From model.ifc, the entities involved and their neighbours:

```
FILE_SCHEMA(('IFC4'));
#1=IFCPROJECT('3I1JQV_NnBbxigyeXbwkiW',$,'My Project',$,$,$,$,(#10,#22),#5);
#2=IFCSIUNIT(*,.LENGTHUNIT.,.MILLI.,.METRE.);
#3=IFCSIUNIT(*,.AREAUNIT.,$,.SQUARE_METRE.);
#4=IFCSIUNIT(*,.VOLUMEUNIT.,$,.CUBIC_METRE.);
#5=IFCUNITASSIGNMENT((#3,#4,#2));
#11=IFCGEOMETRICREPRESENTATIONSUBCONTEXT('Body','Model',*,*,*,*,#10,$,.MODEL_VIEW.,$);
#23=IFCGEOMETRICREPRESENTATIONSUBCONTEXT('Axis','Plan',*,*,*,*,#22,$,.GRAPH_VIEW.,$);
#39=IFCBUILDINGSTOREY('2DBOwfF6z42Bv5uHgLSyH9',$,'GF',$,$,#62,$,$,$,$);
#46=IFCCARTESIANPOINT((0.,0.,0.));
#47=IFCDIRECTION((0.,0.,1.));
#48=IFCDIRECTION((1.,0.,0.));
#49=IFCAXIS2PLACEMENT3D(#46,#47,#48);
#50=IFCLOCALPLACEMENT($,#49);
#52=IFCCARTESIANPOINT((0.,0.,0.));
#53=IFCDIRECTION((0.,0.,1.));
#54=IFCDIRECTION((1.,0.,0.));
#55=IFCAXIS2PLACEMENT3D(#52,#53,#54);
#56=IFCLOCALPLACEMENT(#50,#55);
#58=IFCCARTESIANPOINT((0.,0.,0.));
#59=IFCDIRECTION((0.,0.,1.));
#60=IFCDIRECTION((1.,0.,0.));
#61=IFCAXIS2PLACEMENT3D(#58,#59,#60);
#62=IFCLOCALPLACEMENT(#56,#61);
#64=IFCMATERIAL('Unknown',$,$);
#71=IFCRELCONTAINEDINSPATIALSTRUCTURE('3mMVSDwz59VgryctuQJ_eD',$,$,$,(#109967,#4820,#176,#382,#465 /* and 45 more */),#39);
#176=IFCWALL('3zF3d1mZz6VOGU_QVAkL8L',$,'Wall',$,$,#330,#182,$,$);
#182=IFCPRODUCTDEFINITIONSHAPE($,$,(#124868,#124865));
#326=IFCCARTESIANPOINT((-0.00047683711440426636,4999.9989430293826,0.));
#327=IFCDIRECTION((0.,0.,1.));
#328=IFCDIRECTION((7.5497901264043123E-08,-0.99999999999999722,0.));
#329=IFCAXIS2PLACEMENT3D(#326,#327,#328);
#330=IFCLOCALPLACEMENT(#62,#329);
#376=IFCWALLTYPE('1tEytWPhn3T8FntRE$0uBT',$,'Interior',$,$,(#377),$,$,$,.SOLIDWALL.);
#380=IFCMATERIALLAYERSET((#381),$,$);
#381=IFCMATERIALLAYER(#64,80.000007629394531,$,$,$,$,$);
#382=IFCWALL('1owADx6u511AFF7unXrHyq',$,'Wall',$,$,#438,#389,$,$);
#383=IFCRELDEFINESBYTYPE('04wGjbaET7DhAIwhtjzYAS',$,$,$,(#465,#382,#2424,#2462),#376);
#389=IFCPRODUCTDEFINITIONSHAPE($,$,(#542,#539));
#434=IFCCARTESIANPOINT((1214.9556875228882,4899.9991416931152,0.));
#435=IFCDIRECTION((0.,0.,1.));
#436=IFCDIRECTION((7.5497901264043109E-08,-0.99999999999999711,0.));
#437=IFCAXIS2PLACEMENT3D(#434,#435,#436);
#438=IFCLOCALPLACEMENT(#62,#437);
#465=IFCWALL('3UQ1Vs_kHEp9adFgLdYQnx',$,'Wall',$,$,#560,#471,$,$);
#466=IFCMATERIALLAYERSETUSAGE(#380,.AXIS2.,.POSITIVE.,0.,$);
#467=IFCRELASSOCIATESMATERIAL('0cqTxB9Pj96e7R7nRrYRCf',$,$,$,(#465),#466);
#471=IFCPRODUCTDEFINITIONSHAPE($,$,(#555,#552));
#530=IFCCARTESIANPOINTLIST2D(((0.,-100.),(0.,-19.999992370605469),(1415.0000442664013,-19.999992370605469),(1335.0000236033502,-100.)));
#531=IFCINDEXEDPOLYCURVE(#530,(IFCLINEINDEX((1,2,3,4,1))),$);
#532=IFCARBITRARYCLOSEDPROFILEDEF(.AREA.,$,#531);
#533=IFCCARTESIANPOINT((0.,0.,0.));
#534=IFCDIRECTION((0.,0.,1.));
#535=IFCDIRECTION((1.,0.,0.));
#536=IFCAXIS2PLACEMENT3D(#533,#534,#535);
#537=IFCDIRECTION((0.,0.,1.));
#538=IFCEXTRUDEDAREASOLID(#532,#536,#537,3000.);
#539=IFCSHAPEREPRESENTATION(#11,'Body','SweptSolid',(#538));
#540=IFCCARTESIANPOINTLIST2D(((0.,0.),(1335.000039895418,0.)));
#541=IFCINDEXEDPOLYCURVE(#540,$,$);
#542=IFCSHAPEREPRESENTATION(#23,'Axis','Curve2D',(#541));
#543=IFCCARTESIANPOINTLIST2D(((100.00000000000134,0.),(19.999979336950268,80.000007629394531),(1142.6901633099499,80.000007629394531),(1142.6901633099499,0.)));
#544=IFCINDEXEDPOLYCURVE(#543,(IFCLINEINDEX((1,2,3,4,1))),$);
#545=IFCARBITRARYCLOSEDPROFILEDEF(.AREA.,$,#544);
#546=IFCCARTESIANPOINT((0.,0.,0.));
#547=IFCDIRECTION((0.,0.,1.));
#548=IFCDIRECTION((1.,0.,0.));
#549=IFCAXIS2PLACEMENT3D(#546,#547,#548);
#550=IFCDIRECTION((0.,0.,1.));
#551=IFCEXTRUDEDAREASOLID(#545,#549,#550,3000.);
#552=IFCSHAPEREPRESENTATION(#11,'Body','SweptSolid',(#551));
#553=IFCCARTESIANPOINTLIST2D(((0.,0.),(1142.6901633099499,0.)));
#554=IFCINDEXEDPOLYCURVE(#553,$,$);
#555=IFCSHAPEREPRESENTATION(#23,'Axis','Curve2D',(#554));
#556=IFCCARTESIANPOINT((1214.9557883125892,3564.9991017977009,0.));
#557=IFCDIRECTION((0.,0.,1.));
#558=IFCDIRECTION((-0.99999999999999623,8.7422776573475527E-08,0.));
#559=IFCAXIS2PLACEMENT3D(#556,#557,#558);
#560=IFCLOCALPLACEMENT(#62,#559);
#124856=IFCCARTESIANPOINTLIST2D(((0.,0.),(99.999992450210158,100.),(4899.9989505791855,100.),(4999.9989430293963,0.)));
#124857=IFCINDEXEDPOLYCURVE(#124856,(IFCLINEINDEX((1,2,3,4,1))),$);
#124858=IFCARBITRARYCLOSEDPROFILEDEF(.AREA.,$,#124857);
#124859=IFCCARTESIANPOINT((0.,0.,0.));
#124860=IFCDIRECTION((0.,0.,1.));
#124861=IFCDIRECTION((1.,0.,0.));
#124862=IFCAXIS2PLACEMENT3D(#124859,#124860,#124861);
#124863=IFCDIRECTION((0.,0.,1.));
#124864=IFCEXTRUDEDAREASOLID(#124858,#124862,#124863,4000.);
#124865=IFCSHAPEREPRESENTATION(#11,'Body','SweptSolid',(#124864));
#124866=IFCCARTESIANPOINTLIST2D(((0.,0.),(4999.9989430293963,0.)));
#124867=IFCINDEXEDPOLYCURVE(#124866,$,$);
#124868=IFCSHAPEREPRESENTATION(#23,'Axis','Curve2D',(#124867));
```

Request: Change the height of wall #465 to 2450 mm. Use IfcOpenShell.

```python
import ifcopenshell
import ifcopenshell.geom
import ifcopenshell.util.representation
import ifcopenshell.util.shape
import ifcopenshell.util.unit

model = ifcopenshell.open("model.ifc")
unit_scale = ifcopenshell.util.unit.calculate_unit_scale(model)
settings = ifcopenshell.geom.settings()


def volume(element):
    """Net volume in cubic metres, openings subtracted."""
    shape = ifcopenshell.geom.create_shape(settings, element)
    return ifcopenshell.util.shape.get_volume(shape.geometry)


wall = model.by_id(465)
before = volume(wall)

body = ifcopenshell.util.representation.get_representation(wall, "Model", "Body")
solid = body.Items[0]
old_height = solid.Depth
solid.Depth = 2.45 / unit_scale
after = volume(wall)

print(f"height {old_height:g} -> {solid.Depth:g}, volume {before:.3f} -> {after:.3f} m3")

model.write("model_updated.ifc")
```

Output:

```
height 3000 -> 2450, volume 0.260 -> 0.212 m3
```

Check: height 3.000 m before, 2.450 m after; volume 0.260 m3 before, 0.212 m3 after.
